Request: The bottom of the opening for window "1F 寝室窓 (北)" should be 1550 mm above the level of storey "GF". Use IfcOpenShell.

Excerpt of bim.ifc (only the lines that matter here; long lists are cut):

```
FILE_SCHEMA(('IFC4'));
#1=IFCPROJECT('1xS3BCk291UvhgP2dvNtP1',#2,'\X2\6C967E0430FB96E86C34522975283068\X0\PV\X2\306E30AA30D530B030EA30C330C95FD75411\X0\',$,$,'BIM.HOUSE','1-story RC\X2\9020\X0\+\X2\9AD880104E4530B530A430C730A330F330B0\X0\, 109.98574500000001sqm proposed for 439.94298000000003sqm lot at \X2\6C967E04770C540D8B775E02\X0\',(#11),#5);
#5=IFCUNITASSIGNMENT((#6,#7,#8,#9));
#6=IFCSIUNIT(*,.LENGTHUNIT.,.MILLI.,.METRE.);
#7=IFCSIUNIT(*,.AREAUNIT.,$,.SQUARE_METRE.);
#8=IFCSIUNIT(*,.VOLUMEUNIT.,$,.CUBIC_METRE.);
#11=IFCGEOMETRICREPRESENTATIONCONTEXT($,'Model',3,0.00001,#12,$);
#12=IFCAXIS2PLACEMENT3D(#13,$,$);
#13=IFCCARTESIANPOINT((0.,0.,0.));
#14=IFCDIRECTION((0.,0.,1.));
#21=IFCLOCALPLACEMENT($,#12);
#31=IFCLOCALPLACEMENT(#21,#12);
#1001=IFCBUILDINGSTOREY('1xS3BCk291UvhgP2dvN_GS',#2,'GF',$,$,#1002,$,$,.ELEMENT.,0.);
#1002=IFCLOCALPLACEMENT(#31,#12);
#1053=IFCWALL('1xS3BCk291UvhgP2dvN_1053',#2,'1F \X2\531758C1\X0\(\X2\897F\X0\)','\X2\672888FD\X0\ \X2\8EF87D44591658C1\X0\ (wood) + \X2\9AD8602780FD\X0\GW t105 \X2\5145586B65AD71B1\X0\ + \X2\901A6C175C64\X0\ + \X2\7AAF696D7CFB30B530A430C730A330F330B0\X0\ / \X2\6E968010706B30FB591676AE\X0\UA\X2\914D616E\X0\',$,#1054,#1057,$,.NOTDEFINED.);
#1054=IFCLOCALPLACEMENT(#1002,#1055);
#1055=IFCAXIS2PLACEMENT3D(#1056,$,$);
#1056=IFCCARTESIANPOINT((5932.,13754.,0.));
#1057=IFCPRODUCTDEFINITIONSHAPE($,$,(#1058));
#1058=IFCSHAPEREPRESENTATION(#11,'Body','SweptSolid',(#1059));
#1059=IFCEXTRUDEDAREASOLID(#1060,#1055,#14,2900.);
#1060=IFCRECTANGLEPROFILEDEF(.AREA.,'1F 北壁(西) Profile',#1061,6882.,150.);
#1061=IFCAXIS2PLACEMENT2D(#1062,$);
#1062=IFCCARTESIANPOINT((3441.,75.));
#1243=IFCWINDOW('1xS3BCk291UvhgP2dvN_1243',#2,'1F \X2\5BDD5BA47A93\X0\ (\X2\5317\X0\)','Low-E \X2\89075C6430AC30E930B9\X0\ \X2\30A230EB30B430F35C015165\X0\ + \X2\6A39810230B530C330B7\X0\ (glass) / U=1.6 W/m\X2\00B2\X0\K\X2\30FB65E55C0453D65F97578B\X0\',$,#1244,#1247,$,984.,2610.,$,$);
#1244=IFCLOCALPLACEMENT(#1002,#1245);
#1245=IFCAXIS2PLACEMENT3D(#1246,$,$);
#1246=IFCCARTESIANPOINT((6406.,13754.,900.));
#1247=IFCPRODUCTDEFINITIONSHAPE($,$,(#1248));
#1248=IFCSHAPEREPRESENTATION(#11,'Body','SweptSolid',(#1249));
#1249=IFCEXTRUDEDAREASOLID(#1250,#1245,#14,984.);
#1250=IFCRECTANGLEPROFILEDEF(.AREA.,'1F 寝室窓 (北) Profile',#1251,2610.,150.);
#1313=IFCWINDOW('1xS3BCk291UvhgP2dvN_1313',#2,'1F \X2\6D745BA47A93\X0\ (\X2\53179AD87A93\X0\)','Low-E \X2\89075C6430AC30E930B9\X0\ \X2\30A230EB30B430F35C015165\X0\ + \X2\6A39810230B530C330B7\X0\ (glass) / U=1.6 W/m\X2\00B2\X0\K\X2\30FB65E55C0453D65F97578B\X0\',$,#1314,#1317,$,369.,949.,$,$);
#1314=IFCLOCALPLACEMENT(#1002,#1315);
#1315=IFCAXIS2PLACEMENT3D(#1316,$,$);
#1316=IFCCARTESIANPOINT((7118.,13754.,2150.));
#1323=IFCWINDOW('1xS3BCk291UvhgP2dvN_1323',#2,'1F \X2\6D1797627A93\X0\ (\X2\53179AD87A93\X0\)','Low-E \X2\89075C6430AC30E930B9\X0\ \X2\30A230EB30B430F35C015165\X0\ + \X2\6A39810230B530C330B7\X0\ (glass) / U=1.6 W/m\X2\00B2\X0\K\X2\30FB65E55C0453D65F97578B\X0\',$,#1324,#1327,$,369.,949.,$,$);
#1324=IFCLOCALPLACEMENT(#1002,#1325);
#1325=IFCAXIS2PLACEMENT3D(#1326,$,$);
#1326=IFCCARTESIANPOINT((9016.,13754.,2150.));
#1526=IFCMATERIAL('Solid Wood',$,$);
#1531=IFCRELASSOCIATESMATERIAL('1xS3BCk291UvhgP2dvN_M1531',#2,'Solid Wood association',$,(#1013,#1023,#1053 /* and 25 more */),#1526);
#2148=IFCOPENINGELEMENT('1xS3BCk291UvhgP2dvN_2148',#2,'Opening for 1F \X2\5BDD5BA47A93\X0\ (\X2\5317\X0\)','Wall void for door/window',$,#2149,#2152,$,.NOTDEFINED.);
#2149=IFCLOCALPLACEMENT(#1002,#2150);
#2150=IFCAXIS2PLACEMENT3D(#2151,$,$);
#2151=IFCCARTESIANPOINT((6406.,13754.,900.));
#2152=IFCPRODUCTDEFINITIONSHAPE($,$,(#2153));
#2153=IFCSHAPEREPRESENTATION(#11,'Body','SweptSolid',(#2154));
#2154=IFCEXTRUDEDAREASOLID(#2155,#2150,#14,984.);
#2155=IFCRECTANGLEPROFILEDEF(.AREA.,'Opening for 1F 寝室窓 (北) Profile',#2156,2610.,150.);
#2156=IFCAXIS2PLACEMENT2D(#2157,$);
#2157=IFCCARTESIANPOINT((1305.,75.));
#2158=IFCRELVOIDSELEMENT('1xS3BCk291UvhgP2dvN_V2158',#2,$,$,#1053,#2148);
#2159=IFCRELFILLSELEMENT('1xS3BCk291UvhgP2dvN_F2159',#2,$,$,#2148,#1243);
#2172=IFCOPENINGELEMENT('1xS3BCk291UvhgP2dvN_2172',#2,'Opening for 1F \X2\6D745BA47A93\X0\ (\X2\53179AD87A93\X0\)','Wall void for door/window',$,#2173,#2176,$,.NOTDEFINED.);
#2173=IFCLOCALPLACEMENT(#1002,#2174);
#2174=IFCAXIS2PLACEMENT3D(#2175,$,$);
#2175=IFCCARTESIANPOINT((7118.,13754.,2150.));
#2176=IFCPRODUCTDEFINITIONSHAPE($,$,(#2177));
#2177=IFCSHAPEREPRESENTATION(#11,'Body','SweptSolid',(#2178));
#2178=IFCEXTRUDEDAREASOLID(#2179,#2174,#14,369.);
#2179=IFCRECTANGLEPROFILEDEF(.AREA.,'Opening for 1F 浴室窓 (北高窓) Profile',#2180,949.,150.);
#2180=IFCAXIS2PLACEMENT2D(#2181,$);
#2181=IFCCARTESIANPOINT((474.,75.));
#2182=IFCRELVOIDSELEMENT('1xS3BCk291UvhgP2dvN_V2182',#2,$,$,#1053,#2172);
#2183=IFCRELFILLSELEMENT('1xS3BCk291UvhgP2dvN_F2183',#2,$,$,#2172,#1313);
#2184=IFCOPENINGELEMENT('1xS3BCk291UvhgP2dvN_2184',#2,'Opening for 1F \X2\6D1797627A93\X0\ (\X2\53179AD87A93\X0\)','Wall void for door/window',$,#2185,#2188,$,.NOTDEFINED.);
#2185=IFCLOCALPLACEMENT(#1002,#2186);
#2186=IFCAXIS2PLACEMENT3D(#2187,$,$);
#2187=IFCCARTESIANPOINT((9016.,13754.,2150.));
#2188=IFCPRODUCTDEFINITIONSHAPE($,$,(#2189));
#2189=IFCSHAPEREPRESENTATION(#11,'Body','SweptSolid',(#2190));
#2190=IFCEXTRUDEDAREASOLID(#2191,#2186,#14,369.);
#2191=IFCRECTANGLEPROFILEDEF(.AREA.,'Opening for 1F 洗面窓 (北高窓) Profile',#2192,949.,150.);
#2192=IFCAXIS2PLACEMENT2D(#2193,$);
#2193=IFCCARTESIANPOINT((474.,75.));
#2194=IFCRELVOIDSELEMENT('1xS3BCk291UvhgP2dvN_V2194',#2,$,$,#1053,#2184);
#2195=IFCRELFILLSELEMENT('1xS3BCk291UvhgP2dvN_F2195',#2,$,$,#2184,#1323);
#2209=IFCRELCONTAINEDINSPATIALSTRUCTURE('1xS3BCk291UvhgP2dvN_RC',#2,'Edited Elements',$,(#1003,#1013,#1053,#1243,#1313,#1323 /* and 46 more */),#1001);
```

```python
import numpy as np
import ifcopenshell
import ifcopenshell.api.geometry
import ifcopenshell.geom
import ifcopenshell.util.element
import ifcopenshell.util.placement
import ifcopenshell.util.shape
import ifcopenshell.util.unit

model = ifcopenshell.open("bim.ifc")
unit_scale = ifcopenshell.util.unit.calculate_unit_scale(model)

window = model.by_id(1243)
opening = window.FillsVoids[0].RelatingOpeningElement
storey = ifcopenshell.util.element.get_container(window, ifc_class="IfcBuildingStorey")
level = ifcopenshell.util.placement.get_local_placement(storey.ObjectPlacement)[2, 3]

# The opening's origin need not be at the sill, so measure its lowest point.
shape = ifcopenshell.geom.create_shape(ifcopenshell.geom.settings(), opening)
bottom = ifcopenshell.util.shape.get_shape_bottom_elevation(shape, shape.geometry) / unit_scale
dz = level + 1.55 / unit_scale - bottom

shift = np.array([0.0, 0.0, dz])
# The window is not placed relative to its opening, so move both.
for product in (opening, window):
    matrix = ifcopenshell.util.placement.get_local_placement(product.ObjectPlacement)
    matrix[:3, 3] += shift
    ifcopenshell.api.geometry.edit_object_placement(model, product=product, matrix=matrix, is_si=False)

print(f"moved by {dz * unit_scale:+.3f} m")

model.write("bim_rev.ifc")
```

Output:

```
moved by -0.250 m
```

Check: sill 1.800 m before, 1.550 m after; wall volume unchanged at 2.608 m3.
